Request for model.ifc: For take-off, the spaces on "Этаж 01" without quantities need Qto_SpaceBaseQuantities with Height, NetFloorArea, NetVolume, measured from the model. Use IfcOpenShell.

First a look at what the model holds.

```python
import ifcopenshell
import ifcopenshell.util.element
import ifcopenshell.util.unit

model = ifcopenshell.open("model.ifc")
print(model.schema)
for unit_type in ("LENGTHUNIT", "AREAUNIT", "VOLUMEUNIT"):
    print(unit_type, ifcopenshell.util.unit.calculate_unit_scale(model, unit_type))
storey = next(s for s in model.by_type("IfcBuildingStorey") if s.Name == "Этаж 01")
spaces = [e for e in ifcopenshell.util.element.get_decomposition(storey) if e.is_a("IfcSpace")]
for e in sorted(spaces, key=lambda e: e.id()):
    print(e.id(), e.is_a(), e.Name, list(ifcopenshell.util.element.get_psets(e, qtos_only=True)), sep=" | ")
```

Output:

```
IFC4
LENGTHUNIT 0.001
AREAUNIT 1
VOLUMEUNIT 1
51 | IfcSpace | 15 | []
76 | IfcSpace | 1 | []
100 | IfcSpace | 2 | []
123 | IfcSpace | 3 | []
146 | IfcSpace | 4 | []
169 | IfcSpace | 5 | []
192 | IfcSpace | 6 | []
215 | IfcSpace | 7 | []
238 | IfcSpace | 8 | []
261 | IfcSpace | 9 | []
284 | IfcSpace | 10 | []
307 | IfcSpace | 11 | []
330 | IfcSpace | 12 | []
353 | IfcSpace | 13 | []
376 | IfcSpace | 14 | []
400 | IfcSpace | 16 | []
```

```python
import ifcopenshell
import ifcopenshell.api.pset
import ifcopenshell.geom
import ifcopenshell.util.element
import ifcopenshell.util.shape
import ifcopenshell.util.unit

model = ifcopenshell.open("model.ifc")
unit_scale = ifcopenshell.util.unit.calculate_unit_scale(model)
area_scale = ifcopenshell.util.unit.calculate_unit_scale(model, "AREAUNIT")
volume_scale = ifcopenshell.util.unit.calculate_unit_scale(model, "VOLUMEUNIT")
settings = ifcopenshell.geom.settings()

storey = next(s for s in model.by_type("IfcBuildingStorey") if s.Name == "Этаж 01")
spaces = [e for e in ifcopenshell.util.element.get_decomposition(storey) if e.is_a("IfcSpace")]

for e in sorted(spaces, key=lambda e: e.id()):
    if ifcopenshell.util.element.get_psets(e, qtos_only=True, should_inherit=False):
        continue
    # Geometry comes back in metres, in the element's own axes.
    shape = ifcopenshell.geom.create_shape(settings, e)
    values = {
        "Height": ifcopenshell.util.shape.get_z(shape.geometry) / unit_scale,
        "NetFloorArea": ifcopenshell.util.shape.get_footprint_area(shape.geometry) / area_scale,
        "NetVolume": ifcopenshell.util.shape.get_volume(shape.geometry) / volume_scale,
    }
    qto = ifcopenshell.api.pset.add_qto(model, product=e, name="Qto_SpaceBaseQuantities")
    ifcopenshell.api.pset.edit_qto(model, qto=qto, properties=values)
    print(e.id(), {k: round(v, 3) for k, v in values.items()})

model.write("model_rev.ifc")
```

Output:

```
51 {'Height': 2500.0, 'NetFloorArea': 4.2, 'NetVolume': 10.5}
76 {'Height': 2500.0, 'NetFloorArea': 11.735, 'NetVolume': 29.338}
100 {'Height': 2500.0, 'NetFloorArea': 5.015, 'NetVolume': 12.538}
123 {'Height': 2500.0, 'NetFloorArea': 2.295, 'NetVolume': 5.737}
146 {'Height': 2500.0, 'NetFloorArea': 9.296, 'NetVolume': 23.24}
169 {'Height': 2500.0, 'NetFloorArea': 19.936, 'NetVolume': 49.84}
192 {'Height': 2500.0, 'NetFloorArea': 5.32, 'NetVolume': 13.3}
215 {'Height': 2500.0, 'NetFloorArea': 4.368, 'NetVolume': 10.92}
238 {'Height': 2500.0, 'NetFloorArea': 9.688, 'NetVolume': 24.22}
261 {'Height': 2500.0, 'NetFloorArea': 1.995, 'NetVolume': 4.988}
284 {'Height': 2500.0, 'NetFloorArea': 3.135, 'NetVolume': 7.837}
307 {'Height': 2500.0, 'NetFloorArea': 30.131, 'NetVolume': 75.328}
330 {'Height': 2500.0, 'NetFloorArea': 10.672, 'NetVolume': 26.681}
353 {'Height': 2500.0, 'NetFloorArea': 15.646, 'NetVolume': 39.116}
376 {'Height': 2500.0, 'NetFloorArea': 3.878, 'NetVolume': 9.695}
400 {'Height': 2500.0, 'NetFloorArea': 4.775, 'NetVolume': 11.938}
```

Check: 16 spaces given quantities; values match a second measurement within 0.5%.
